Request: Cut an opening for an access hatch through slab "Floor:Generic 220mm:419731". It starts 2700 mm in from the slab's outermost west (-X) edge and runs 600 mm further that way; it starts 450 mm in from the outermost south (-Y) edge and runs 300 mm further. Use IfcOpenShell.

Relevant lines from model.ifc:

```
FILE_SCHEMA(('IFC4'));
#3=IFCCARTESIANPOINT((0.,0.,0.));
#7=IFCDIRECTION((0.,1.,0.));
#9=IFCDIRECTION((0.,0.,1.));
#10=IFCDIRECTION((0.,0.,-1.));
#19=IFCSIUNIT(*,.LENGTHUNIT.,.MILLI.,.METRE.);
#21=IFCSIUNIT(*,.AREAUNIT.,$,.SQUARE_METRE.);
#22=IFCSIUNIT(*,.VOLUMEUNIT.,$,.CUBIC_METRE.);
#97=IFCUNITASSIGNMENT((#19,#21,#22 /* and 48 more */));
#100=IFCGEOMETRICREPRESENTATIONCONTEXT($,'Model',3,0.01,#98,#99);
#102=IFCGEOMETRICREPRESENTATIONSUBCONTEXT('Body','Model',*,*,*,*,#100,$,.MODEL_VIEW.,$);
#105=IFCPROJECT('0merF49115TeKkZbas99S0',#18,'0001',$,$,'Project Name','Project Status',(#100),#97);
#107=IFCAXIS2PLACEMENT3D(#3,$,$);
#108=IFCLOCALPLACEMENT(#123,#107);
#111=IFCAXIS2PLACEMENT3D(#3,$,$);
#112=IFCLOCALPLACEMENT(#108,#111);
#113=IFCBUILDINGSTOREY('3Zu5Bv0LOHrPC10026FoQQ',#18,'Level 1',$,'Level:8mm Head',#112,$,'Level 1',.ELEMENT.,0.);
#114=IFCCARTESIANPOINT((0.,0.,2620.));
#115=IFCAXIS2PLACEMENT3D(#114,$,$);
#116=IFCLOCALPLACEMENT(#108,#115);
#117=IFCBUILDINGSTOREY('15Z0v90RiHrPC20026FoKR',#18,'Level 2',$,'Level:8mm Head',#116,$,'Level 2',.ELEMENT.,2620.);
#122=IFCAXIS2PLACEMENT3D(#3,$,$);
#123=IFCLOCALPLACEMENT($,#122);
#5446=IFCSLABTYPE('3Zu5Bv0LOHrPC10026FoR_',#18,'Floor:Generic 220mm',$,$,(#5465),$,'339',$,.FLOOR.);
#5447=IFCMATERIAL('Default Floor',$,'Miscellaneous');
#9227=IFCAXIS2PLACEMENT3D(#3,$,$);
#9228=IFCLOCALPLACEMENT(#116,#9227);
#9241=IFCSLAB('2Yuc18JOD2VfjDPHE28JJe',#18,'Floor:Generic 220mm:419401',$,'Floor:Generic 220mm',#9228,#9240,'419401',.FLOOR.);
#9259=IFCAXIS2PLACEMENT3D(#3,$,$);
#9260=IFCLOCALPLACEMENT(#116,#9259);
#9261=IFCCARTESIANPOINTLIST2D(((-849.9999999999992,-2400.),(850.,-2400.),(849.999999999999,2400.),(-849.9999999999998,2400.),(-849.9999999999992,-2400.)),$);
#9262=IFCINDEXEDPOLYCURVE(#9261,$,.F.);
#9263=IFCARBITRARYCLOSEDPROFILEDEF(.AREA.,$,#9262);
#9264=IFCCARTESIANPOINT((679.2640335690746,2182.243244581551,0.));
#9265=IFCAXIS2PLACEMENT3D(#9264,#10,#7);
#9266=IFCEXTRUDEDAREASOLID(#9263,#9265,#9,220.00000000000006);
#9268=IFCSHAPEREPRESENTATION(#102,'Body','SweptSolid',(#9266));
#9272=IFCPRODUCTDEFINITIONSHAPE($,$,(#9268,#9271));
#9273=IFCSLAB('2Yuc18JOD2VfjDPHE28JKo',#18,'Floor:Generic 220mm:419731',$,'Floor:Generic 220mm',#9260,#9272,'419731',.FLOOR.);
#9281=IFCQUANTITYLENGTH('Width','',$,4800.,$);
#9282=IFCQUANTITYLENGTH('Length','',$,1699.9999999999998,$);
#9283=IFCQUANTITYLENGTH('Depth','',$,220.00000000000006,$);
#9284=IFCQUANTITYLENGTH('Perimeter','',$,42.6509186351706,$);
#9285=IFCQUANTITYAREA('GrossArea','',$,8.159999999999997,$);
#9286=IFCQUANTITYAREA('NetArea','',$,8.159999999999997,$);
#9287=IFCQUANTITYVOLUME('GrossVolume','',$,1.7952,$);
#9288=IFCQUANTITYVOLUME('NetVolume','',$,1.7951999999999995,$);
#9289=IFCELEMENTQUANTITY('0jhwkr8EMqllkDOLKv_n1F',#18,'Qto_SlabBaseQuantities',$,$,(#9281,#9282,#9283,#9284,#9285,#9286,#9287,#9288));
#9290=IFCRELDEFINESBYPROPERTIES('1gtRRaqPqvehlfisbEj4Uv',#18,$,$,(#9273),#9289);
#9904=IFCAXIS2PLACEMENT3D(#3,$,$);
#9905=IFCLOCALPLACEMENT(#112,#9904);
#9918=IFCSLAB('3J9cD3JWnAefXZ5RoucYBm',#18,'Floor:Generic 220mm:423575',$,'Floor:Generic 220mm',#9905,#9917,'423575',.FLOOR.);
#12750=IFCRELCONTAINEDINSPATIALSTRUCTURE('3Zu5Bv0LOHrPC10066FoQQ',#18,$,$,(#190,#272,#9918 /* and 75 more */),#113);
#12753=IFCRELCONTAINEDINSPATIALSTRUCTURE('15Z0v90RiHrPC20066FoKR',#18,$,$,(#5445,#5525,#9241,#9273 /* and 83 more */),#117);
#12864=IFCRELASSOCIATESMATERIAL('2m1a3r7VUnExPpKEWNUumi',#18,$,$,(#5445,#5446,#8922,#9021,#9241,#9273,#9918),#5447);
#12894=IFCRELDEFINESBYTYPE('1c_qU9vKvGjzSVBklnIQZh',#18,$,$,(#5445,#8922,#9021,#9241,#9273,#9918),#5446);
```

```python
import numpy as np
import ifcopenshell
import ifcopenshell.api.feature
import ifcopenshell.api.geometry
import ifcopenshell.api.pset
import ifcopenshell.api.root
import ifcopenshell.geom
import ifcopenshell.util.element
import ifcopenshell.util.placement
import ifcopenshell.util.representation
import ifcopenshell.util.shape
import ifcopenshell.util.unit

model = ifcopenshell.open("model.ifc")
unit_scale = ifcopenshell.util.unit.calculate_unit_scale(model)
area_scale = ifcopenshell.util.unit.calculate_unit_scale(model, "AREAUNIT")
volume_scale = ifcopenshell.util.unit.calculate_unit_scale(model, "VOLUMEUNIT")
settings = ifcopenshell.geom.settings()


def volume(element):
    """Net volume in cubic metres, openings subtracted."""
    shape = ifcopenshell.geom.create_shape(settings, element)
    return ifcopenshell.util.shape.get_volume(shape.geometry)


slab = model.by_guid("2Yuc18JOD2VfjDPHE28JKo")
before = volume(slab)

# Extent in the slab's own axes, in metres. The edges named are its -X and -Y sides.
slab_shape = ifcopenshell.geom.create_shape(settings, slab)
vertices = ifcopenshell.util.shape.get_vertices(slab_shape.geometry)
x_min, y_min, bottom = vertices.min(axis=0)
top = vertices[:, 2].max()

opening = ifcopenshell.api.root.create_entity(model, ifc_class="IfcOpeningElement", name="Access hatch opening", predefined_type="OPENING")
context = ifcopenshell.util.representation.get_context(model, "Model", "Body", "MODEL_VIEW")
width, depth = 0.6, 0.3
outline = [(0.0, 0.0), (width, 0.0), (width, depth), (0.0, depth), (0.0, 0.0)]
# Overshoot both faces by 50 mm so the cut is clean.
shape = ifcopenshell.api.geometry.add_slab_representation(
    model, context=context, depth=top - bottom + 0.1, polyline=outline
)
ifcopenshell.api.geometry.assign_representation(model, product=opening, representation=shape)

matrix = ifcopenshell.util.placement.get_local_placement(slab.ObjectPlacement)
matrix[:, 3] = matrix @ np.append(np.array([x_min + 2.7, y_min + 0.45, bottom - 0.05]) / unit_scale, 1.0)
ifcopenshell.api.geometry.edit_object_placement(model, product=opening, matrix=matrix, is_si=False)
ifcopenshell.api.feature.add_feature(model, feature=opening, element=slab)

after = volume(slab)

# Update the slab's stored quantities.
qto = model.by_id(ifcopenshell.util.element.get_pset(slab, "Qto_SlabBaseQuantities", should_inherit=False)["id"])
ifcopenshell.api.pset.edit_qto(model, qto=qto, properties={
    "NetArea": after / (top - bottom) / area_scale,
    "NetVolume": after / volume_scale,
})

print(f"slab volume {before:.3f} -> {after:.3f} m3")

model.write("model_updated.ifc")
```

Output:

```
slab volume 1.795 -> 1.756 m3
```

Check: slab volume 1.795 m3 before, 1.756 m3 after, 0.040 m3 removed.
